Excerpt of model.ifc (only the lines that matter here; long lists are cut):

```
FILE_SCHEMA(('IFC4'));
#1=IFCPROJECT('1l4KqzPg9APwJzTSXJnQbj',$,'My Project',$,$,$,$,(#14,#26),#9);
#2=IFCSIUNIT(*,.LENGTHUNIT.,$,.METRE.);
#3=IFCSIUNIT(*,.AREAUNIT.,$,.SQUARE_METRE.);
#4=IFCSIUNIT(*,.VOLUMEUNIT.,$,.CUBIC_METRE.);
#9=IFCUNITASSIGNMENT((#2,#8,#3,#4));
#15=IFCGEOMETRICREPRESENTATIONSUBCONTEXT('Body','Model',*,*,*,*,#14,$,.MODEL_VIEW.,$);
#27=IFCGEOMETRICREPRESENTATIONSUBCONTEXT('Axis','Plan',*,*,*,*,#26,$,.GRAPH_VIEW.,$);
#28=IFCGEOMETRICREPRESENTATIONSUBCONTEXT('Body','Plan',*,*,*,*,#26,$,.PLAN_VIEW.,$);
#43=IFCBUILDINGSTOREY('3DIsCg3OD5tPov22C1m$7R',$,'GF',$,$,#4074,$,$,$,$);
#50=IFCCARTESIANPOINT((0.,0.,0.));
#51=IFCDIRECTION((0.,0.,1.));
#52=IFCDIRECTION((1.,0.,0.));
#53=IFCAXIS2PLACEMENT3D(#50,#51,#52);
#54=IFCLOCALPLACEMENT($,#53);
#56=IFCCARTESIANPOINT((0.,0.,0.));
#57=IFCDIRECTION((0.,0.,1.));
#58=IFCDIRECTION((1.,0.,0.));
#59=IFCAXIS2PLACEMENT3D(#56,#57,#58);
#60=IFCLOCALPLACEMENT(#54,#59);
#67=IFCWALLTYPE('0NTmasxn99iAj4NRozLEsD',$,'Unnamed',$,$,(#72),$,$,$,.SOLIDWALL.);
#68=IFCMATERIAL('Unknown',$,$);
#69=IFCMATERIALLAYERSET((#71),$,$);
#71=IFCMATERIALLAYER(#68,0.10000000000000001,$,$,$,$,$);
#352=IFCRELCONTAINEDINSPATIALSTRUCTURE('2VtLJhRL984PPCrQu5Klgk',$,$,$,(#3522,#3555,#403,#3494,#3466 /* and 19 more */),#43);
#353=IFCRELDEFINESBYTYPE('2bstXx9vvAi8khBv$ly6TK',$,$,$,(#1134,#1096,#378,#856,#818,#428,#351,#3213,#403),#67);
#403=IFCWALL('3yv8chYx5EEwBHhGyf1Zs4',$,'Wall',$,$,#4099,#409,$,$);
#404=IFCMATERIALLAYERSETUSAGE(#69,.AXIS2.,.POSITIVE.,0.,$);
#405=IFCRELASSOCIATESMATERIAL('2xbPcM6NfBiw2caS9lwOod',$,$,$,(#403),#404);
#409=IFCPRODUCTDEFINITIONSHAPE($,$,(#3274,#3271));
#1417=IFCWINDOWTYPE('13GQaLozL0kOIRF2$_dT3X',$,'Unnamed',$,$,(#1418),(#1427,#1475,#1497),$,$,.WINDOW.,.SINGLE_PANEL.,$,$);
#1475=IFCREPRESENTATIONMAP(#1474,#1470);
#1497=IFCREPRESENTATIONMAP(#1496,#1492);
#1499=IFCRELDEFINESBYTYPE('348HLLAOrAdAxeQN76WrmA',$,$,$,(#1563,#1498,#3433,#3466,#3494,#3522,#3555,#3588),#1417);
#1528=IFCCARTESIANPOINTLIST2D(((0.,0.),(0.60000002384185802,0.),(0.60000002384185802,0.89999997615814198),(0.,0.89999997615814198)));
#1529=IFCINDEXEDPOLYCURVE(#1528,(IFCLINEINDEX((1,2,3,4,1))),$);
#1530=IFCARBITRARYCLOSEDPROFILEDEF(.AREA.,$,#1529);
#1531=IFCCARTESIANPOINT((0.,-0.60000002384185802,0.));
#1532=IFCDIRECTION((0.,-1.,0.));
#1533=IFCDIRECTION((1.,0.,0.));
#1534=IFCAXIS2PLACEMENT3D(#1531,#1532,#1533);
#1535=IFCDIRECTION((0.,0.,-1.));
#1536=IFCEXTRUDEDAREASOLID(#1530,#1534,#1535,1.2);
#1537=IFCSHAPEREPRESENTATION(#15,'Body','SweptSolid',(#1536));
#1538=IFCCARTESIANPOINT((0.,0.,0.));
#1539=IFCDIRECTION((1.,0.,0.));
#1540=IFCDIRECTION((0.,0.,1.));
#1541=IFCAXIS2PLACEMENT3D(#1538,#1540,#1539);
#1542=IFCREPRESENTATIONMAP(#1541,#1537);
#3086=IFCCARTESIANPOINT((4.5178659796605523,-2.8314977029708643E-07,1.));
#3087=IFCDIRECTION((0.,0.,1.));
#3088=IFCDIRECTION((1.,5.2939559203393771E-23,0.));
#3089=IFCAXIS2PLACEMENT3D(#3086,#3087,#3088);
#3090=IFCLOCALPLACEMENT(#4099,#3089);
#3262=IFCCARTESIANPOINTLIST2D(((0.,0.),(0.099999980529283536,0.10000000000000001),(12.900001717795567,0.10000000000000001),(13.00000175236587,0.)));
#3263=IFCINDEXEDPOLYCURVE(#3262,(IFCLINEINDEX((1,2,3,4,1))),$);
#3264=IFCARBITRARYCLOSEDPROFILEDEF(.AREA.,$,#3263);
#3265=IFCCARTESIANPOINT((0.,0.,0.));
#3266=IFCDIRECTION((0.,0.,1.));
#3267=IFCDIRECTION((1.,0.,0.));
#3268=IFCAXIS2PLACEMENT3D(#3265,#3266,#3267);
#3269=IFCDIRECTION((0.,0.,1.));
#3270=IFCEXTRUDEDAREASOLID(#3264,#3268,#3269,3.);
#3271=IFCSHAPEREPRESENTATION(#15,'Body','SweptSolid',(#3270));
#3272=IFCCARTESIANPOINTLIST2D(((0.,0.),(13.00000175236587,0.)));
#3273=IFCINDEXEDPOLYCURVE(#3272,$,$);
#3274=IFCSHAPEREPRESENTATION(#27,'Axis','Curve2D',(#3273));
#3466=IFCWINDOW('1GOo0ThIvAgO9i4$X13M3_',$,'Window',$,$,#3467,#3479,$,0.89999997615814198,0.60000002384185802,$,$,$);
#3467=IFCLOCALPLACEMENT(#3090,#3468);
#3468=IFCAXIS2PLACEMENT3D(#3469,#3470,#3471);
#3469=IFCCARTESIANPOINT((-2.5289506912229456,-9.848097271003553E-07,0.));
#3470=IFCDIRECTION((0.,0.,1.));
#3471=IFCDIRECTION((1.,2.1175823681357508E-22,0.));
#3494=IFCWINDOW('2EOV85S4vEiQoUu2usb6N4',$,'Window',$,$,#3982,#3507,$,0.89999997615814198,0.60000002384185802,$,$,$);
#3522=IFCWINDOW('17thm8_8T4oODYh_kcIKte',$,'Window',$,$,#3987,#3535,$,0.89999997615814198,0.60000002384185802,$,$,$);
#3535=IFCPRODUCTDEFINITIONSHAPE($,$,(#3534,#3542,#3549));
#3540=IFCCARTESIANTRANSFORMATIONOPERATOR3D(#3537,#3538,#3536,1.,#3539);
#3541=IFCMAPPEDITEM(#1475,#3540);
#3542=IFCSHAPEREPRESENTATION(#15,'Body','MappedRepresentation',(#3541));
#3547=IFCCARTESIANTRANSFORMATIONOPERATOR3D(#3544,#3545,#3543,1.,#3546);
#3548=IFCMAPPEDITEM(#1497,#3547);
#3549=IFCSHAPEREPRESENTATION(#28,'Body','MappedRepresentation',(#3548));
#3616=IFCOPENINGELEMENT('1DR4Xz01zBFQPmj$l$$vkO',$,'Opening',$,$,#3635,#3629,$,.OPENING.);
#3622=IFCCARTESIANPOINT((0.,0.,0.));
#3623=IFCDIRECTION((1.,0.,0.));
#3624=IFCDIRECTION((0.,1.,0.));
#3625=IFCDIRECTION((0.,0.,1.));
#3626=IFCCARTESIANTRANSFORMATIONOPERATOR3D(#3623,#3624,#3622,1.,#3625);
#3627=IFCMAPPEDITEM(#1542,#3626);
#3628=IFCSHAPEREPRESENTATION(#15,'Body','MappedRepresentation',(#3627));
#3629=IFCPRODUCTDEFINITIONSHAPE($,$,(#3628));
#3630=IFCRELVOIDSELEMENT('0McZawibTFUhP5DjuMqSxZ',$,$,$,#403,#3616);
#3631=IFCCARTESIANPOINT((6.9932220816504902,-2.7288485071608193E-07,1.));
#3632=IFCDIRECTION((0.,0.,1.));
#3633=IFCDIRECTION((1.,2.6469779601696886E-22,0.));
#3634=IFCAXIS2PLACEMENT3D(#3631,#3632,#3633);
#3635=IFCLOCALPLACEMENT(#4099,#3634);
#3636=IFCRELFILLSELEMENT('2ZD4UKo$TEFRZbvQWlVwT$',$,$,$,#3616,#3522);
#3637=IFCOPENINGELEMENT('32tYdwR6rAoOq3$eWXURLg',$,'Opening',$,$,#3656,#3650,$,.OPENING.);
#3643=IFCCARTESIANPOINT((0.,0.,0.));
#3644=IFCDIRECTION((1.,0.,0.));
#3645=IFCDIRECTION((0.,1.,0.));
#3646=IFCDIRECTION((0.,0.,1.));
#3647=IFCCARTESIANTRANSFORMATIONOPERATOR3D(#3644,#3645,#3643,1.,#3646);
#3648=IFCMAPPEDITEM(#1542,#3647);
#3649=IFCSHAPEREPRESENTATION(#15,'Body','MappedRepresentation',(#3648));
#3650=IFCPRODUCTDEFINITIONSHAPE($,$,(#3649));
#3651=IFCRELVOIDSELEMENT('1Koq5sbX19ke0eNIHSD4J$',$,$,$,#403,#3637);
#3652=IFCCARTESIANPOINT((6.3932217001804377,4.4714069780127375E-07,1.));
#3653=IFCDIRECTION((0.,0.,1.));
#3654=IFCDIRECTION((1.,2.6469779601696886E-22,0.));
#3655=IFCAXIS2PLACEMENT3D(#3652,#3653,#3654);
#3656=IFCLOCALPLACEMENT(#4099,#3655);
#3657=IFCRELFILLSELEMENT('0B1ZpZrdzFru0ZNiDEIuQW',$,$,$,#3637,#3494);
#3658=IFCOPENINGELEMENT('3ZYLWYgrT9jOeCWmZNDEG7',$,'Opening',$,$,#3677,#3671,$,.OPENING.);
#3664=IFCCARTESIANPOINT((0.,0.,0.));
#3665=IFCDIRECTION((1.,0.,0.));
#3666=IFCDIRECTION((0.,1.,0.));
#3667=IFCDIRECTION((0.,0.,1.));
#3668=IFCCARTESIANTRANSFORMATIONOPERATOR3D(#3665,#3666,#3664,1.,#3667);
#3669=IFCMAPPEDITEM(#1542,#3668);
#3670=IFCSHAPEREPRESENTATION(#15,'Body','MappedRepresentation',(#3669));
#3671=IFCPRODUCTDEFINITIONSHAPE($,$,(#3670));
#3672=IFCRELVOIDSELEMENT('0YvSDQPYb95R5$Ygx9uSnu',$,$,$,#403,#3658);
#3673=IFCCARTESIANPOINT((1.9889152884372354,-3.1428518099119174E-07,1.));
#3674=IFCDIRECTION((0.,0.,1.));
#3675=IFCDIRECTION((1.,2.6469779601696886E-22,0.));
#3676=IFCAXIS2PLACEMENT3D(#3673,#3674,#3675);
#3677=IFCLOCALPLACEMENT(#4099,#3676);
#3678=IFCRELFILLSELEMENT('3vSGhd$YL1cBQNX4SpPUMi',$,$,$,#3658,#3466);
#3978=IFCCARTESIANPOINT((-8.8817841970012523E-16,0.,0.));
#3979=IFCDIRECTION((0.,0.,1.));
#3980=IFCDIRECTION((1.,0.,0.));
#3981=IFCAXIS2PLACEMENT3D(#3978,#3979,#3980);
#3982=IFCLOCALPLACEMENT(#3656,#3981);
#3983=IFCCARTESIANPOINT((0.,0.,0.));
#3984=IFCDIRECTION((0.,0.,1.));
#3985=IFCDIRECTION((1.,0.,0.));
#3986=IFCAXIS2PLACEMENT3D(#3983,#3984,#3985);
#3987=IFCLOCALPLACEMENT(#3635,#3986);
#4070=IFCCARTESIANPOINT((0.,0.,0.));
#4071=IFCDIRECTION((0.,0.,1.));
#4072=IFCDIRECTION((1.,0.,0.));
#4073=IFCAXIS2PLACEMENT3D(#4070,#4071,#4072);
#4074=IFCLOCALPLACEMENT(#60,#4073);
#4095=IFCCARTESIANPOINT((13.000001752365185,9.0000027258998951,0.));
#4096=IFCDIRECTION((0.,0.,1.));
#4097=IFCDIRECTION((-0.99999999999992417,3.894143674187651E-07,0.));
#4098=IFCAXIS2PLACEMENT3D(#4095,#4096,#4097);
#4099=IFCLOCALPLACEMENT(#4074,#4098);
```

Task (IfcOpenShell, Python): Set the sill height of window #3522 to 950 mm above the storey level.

```python
import numpy as np
import ifcopenshell
import ifcopenshell.api.geometry
import ifcopenshell.geom
import ifcopenshell.util.element
import ifcopenshell.util.placement
import ifcopenshell.util.shape
import ifcopenshell.util.unit

model = ifcopenshell.open("model.ifc")
unit_scale = ifcopenshell.util.unit.calculate_unit_scale(model)

window = model.by_id(3522)
opening = window.FillsVoids[0].RelatingOpeningElement
storey = ifcopenshell.util.element.get_container(window, ifc_class="IfcBuildingStorey")
level = ifcopenshell.util.placement.get_local_placement(storey.ObjectPlacement)[2, 3]

# The opening's origin need not be at the sill, so measure its lowest point.
shape = ifcopenshell.geom.create_shape(ifcopenshell.geom.settings(), opening)
bottom = ifcopenshell.util.shape.get_shape_bottom_elevation(shape, shape.geometry) / unit_scale
dz = level + 0.95 / unit_scale - bottom

shift = np.array([0.0, 0.0, dz])
# The window is placed relative to its opening, so it follows when the opening moves.
matrix = ifcopenshell.util.placement.get_local_placement(opening.ObjectPlacement)
matrix[:3, 3] += shift
ifcopenshell.api.geometry.edit_object_placement(
    model, product=opening, matrix=matrix, is_si=False, should_transform_children=True
)

print(f"moved by {dz * unit_scale:+.3f} m")

model.write("model-out.ifc")
```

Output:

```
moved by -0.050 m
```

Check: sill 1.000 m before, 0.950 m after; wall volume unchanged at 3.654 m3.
